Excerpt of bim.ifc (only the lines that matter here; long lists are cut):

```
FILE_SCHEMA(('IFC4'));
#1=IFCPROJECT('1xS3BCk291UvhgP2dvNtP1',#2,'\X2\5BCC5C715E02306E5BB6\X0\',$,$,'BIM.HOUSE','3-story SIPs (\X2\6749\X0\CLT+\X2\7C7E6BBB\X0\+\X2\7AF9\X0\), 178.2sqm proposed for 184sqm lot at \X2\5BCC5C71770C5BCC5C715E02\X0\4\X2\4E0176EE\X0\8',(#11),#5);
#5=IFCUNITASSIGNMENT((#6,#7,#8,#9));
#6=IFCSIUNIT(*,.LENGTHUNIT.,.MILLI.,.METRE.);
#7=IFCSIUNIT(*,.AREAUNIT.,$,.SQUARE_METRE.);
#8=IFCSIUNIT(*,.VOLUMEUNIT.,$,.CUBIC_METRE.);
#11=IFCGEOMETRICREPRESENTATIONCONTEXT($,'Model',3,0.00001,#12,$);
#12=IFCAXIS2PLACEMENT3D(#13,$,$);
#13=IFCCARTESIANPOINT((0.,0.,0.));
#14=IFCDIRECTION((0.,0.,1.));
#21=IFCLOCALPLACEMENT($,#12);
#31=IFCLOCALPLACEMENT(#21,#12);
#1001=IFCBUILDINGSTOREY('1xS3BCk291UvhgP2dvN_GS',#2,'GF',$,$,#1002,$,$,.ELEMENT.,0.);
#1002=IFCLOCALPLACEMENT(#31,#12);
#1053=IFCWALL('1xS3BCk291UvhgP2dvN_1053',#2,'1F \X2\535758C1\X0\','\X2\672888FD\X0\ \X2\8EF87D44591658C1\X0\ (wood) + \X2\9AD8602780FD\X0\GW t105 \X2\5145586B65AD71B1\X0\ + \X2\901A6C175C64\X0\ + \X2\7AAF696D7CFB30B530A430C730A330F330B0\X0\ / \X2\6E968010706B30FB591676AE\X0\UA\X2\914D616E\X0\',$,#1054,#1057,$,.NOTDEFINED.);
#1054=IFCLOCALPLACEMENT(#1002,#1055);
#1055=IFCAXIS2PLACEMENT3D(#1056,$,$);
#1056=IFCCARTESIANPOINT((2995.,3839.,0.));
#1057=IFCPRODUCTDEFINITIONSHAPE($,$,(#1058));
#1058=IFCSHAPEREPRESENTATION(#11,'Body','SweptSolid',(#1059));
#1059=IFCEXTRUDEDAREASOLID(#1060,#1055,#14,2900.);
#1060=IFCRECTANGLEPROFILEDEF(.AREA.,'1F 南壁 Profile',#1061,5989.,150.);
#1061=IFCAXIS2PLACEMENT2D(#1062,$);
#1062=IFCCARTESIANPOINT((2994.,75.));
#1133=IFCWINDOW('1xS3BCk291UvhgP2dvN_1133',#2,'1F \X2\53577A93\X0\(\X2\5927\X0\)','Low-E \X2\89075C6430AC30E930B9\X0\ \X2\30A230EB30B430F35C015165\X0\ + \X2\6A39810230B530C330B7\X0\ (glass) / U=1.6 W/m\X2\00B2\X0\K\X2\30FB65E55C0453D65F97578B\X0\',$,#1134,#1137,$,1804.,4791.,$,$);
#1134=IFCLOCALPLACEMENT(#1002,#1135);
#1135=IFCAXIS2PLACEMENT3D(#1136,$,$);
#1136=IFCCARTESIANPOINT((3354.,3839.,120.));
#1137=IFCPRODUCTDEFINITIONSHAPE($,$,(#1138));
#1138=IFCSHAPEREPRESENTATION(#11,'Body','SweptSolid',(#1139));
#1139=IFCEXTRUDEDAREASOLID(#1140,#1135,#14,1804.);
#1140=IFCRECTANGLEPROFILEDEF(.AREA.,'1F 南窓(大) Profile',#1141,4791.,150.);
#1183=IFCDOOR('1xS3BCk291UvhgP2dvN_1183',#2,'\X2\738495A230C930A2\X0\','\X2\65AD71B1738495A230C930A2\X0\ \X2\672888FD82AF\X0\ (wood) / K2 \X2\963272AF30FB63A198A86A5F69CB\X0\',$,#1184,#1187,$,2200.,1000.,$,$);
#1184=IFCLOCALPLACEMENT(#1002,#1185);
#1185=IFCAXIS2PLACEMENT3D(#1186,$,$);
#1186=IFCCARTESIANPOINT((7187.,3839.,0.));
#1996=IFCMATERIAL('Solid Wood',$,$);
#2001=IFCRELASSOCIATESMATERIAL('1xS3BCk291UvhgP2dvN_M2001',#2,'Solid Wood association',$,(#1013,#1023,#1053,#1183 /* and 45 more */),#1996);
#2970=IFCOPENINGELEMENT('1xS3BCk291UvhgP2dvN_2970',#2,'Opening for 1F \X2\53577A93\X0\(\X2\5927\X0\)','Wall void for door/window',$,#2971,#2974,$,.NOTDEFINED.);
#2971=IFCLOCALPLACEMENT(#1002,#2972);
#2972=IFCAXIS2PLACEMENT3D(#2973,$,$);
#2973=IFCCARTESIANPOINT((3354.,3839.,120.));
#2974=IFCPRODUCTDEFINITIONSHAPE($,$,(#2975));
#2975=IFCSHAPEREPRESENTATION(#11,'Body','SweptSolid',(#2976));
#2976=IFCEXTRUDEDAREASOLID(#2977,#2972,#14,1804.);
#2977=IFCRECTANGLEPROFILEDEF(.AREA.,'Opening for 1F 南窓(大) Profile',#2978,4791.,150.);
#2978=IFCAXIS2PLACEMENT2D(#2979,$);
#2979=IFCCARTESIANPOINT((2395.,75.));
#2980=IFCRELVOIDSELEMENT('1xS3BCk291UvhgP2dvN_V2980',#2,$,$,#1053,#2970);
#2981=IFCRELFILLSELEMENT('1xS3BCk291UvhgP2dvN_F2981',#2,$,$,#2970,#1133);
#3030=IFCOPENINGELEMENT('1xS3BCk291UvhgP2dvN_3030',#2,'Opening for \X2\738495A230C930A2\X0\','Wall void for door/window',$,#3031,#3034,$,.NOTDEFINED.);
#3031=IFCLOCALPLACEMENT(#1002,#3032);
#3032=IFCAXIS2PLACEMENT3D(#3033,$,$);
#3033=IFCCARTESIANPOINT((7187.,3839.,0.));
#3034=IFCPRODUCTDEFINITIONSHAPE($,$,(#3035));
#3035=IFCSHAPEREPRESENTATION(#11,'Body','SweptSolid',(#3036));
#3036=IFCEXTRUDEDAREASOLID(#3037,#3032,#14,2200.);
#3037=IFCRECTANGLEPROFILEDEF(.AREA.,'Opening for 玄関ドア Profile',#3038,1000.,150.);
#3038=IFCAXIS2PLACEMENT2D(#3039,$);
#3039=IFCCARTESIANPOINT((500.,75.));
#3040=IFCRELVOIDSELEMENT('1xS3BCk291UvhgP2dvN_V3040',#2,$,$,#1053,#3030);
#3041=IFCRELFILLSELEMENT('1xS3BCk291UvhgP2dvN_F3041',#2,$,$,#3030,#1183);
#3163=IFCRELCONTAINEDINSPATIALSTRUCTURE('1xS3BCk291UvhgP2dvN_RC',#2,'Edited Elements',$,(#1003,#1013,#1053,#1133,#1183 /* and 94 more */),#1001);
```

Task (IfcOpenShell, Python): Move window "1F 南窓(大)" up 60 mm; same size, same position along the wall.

```python
import numpy as np
import ifcopenshell
import ifcopenshell.api.geometry
import ifcopenshell.util.placement
import ifcopenshell.util.unit

model = ifcopenshell.open("bim.ifc")
unit_scale = ifcopenshell.util.unit.calculate_unit_scale(model)

window = model.by_id(1133)
opening = window.FillsVoids[0].RelatingOpeningElement
dz = 60.0

shift = np.array([0.0, 0.0, dz])
# The window is not placed relative to its opening, so move both.
for product in (opening, window):
    matrix = ifcopenshell.util.placement.get_local_placement(product.ObjectPlacement)
    matrix[:3, 3] += shift
    ifcopenshell.api.geometry.edit_object_placement(model, product=product, matrix=matrix, is_si=False)

print(f"moved by {dz * unit_scale:+.3f} m")

model.write("bim_rev.ifc")
```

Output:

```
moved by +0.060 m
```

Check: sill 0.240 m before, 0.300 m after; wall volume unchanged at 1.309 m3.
